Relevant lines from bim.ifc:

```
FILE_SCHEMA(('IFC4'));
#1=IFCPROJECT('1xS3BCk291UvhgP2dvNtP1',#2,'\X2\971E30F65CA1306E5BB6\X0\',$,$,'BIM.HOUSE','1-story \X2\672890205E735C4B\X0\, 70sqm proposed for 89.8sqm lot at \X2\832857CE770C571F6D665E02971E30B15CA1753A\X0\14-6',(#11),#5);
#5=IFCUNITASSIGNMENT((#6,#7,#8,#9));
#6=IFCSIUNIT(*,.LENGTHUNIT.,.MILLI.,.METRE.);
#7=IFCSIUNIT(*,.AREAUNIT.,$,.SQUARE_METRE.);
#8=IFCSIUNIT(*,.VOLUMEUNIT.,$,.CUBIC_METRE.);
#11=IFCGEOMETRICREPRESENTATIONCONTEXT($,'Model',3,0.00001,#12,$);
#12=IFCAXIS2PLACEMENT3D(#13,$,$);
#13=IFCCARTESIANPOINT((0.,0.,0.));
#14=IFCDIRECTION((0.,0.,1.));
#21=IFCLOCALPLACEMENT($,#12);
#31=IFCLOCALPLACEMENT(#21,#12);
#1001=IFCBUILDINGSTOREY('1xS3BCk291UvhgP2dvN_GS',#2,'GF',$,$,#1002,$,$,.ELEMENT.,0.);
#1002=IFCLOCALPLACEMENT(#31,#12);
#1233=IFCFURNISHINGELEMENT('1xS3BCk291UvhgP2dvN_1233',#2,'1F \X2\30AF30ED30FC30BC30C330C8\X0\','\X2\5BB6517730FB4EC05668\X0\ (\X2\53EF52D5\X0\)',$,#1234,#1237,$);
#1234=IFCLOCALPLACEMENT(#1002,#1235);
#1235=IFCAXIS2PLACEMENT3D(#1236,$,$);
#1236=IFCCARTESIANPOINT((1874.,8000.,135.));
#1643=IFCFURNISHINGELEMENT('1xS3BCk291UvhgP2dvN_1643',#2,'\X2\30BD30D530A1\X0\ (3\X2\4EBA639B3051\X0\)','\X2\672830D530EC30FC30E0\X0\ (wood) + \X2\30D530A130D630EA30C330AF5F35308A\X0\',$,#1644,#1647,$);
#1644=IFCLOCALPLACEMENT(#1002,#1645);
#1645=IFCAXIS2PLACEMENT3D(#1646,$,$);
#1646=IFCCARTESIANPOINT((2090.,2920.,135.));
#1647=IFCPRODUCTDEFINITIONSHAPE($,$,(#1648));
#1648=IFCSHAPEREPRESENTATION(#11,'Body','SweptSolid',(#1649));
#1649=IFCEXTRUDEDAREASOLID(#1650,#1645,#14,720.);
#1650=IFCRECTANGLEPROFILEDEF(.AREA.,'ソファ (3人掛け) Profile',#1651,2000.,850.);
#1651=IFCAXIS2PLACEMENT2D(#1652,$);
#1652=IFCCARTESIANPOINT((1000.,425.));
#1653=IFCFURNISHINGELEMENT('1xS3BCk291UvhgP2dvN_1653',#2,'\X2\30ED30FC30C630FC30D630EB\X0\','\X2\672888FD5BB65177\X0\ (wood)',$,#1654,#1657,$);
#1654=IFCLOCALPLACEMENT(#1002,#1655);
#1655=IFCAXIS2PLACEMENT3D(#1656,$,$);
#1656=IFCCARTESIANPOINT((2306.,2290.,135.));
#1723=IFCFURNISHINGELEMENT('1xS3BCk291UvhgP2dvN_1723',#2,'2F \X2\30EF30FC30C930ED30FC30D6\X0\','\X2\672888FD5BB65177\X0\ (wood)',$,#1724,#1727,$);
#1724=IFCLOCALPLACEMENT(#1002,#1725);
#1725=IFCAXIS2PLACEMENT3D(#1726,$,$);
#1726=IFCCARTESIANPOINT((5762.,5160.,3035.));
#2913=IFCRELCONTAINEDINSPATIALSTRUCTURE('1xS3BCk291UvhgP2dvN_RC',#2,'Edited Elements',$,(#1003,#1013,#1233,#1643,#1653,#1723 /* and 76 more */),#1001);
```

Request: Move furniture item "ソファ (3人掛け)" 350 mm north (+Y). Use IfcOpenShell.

```python
import ifcopenshell
import ifcopenshell.api.geometry
import ifcopenshell.util.placement
import ifcopenshell.util.unit

model = ifcopenshell.open("bim.ifc")
unit_scale = ifcopenshell.util.unit.calculate_unit_scale(model)

item = model.by_guid("1xS3BCk291UvhgP2dvN_1643")
matrix = ifcopenshell.util.placement.get_local_placement(item.ObjectPlacement)
matrix[1, 3] += 0.35 / unit_scale
ifcopenshell.api.geometry.edit_object_placement(model, product=item, matrix=matrix, is_si=False)

print(ifcopenshell.util.placement.get_local_placement(item.ObjectPlacement).round(3) + 0.0)

model.write("bim_rev.ifc")
```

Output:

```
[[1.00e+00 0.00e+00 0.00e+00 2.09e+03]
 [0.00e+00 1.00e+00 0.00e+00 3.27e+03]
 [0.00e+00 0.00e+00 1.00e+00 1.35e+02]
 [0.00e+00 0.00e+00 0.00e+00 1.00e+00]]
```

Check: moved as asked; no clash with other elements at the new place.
